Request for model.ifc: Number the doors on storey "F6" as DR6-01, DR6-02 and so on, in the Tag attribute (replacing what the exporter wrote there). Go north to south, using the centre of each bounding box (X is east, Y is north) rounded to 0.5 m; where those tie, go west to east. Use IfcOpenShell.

First a look at what the model holds.

```python
import ifcopenshell
import ifcopenshell.util.element
import ifcopenshell.util.placement

model = ifcopenshell.open("model.ifc")
print(model.schema)
storey = next(s for s in model.by_type("IfcBuildingStorey") if s.Name == "F6")
doors = [e for e in ifcopenshell.util.element.get_decomposition(storey) if e.is_a("IfcDoor")]
for e in sorted(doors, key=lambda e: e.id()):
    origin = ifcopenshell.util.placement.get_local_placement(e.ObjectPlacement)[:3, 3]
    print(e.id(), e.Tag, e.Name, origin.round(2) + 0.0, sep=" | ")
```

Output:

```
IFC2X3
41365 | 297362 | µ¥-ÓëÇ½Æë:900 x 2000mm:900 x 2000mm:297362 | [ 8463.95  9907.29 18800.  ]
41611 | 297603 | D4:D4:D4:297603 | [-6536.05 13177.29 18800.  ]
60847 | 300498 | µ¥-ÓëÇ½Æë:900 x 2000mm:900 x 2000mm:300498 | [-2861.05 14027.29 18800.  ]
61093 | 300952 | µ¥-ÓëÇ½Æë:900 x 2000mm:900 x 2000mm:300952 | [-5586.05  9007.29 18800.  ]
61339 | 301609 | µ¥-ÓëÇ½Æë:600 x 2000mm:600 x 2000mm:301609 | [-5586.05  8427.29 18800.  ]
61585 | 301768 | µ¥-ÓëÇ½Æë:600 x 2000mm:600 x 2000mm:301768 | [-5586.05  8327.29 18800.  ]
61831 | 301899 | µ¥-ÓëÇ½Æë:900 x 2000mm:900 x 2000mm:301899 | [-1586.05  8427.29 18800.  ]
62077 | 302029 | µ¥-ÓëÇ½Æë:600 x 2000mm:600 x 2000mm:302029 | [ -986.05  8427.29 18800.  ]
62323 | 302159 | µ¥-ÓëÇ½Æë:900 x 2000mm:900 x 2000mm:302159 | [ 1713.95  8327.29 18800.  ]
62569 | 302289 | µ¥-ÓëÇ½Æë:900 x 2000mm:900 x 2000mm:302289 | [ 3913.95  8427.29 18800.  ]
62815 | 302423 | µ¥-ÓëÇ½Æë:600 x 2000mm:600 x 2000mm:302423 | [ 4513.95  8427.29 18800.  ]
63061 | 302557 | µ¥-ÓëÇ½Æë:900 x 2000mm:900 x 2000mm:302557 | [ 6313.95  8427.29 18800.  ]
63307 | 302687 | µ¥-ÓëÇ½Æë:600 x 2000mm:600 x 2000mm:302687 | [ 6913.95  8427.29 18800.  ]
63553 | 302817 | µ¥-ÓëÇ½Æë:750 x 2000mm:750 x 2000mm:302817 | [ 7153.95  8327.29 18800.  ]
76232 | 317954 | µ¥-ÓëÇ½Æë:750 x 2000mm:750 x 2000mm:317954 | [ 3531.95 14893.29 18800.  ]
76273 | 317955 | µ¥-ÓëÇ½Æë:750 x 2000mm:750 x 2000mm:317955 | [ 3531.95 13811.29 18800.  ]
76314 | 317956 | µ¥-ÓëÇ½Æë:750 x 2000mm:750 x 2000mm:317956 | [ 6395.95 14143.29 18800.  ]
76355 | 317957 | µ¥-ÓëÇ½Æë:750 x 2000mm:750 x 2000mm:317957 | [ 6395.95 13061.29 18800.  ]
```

```python
import ifcopenshell
import ifcopenshell.geom
import ifcopenshell.util.element
import ifcopenshell.util.shape

model = ifcopenshell.open("model.ifc")
settings = ifcopenshell.geom.settings()
settings.set("use-world-coords", True)


def centre(element):
    shape = ifcopenshell.geom.create_shape(settings, element)
    return ifcopenshell.util.shape.get_bbox_centroid(shape.geometry)


storey = next(s for s in model.by_type("IfcBuildingStorey") if s.Name == "F6")
doors = [e for e in ifcopenshell.util.element.get_decomposition(storey) if e.is_a("IfcDoor")]

# Insertion points can sit at a corner or the storey origin, so sort by the geometry (in metres).
centres = {e: centre(e) for e in doors}
doors.sort(key=lambda e: (-round(centres[e][1] / 0.5), centres[e][0]))

for i, e in enumerate(doors, start=1):
    number = f"DR6-{i:02d}"
    e.Tag = number
    print(e.id(), number)

model.write("model_v2.ifc")
```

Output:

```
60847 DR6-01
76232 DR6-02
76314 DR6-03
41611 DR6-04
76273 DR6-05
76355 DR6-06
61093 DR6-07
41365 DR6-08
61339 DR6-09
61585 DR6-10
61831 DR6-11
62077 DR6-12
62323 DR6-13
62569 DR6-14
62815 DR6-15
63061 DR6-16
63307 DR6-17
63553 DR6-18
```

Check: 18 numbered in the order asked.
